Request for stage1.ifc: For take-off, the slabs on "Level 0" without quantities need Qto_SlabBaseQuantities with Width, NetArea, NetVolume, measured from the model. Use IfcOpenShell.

First a look at what the model holds.

```python
import ifcopenshell
import ifcopenshell.util.element
import ifcopenshell.util.unit

model = ifcopenshell.open("stage1.ifc")
print(model.schema)
for unit_type in ("LENGTHUNIT", "AREAUNIT", "VOLUMEUNIT"):
    print(unit_type, ifcopenshell.util.unit.calculate_unit_scale(model, unit_type))
storey = next(s for s in model.by_type("IfcBuildingStorey") if s.Name == "Level 0")
slabs = [e for e in ifcopenshell.util.element.get_decomposition(storey) if e.is_a("IfcSlab")]
for e in sorted(slabs, key=lambda e: e.id()):
    print(e.id(), e.is_a(), e.Name, list(ifcopenshell.util.element.get_psets(e, qtos_only=True)), sep=" | ")
```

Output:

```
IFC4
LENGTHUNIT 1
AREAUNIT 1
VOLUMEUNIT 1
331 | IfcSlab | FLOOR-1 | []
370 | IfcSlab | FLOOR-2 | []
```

```python
import ifcopenshell
import ifcopenshell.api.pset
import ifcopenshell.geom
import ifcopenshell.util.element
import ifcopenshell.util.shape
import ifcopenshell.util.unit

model = ifcopenshell.open("stage1.ifc")
unit_scale = ifcopenshell.util.unit.calculate_unit_scale(model)
area_scale = ifcopenshell.util.unit.calculate_unit_scale(model, "AREAUNIT")
volume_scale = ifcopenshell.util.unit.calculate_unit_scale(model, "VOLUMEUNIT")
settings = ifcopenshell.geom.settings()

storey = next(s for s in model.by_type("IfcBuildingStorey") if s.Name == "Level 0")
slabs = [e for e in ifcopenshell.util.element.get_decomposition(storey) if e.is_a("IfcSlab")]

for e in sorted(slabs, key=lambda e: e.id()):
    if ifcopenshell.util.element.get_psets(e, qtos_only=True, should_inherit=False):
        continue
    # Geometry comes back in metres, in the element's own axes.
    shape = ifcopenshell.geom.create_shape(settings, e)
    values = {
        "Width": ifcopenshell.util.shape.get_z(shape.geometry) / unit_scale,
        "NetArea": ifcopenshell.util.shape.get_footprint_area(shape.geometry) / area_scale,
        "NetVolume": ifcopenshell.util.shape.get_volume(shape.geometry) / volume_scale,
    }
    qto = ifcopenshell.api.pset.add_qto(model, product=e, name="Qto_SlabBaseQuantities")
    ifcopenshell.api.pset.edit_qto(model, qto=qto, properties=values)
    print(e.id(), {k: round(v, 3) for k, v in values.items()})

model.write("stage1_edited.ifc")
```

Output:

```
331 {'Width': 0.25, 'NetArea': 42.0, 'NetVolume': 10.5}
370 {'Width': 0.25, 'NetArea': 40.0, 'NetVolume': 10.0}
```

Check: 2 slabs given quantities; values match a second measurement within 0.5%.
